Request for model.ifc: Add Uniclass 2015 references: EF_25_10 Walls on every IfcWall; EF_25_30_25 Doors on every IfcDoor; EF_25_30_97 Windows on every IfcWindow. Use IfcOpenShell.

First a look at what the model holds.

```python
import ifcopenshell

model = ifcopenshell.open("model.ifc")
print(model.schema)
print("classifications:", [c.Name for c in model.by_type("IfcClassification")])
for ifc_class in ("IfcDoor", "IfcRoof", "IfcStair", "IfcWall", "IfcWindow"):
    print(ifc_class, len(model.by_type(ifc_class)))
```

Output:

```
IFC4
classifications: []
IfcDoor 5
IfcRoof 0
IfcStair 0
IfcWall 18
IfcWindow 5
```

```python
import ifcopenshell
import ifcopenshell.api.classification

model = ifcopenshell.open("model.ifc")

system = ifcopenshell.api.classification.add_classification(model, classification="Uniclass 2015")

codes = {
    "IfcWall": ("EF_25_10", "Walls"),
    "IfcDoor": ("EF_25_30_25", "Doors"),
    "IfcWindow": ("EF_25_30_97", "Windows"),
}
for ifc_class, (code, name) in codes.items():
    products = model.by_type(ifc_class)
    ifcopenshell.api.classification.add_reference(
        model, products=products, classification=system, identification=code, name=name
    )
    print(code, len(products))

model.write("model_rev.ifc")
```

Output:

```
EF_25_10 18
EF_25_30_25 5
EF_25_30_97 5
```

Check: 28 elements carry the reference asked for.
